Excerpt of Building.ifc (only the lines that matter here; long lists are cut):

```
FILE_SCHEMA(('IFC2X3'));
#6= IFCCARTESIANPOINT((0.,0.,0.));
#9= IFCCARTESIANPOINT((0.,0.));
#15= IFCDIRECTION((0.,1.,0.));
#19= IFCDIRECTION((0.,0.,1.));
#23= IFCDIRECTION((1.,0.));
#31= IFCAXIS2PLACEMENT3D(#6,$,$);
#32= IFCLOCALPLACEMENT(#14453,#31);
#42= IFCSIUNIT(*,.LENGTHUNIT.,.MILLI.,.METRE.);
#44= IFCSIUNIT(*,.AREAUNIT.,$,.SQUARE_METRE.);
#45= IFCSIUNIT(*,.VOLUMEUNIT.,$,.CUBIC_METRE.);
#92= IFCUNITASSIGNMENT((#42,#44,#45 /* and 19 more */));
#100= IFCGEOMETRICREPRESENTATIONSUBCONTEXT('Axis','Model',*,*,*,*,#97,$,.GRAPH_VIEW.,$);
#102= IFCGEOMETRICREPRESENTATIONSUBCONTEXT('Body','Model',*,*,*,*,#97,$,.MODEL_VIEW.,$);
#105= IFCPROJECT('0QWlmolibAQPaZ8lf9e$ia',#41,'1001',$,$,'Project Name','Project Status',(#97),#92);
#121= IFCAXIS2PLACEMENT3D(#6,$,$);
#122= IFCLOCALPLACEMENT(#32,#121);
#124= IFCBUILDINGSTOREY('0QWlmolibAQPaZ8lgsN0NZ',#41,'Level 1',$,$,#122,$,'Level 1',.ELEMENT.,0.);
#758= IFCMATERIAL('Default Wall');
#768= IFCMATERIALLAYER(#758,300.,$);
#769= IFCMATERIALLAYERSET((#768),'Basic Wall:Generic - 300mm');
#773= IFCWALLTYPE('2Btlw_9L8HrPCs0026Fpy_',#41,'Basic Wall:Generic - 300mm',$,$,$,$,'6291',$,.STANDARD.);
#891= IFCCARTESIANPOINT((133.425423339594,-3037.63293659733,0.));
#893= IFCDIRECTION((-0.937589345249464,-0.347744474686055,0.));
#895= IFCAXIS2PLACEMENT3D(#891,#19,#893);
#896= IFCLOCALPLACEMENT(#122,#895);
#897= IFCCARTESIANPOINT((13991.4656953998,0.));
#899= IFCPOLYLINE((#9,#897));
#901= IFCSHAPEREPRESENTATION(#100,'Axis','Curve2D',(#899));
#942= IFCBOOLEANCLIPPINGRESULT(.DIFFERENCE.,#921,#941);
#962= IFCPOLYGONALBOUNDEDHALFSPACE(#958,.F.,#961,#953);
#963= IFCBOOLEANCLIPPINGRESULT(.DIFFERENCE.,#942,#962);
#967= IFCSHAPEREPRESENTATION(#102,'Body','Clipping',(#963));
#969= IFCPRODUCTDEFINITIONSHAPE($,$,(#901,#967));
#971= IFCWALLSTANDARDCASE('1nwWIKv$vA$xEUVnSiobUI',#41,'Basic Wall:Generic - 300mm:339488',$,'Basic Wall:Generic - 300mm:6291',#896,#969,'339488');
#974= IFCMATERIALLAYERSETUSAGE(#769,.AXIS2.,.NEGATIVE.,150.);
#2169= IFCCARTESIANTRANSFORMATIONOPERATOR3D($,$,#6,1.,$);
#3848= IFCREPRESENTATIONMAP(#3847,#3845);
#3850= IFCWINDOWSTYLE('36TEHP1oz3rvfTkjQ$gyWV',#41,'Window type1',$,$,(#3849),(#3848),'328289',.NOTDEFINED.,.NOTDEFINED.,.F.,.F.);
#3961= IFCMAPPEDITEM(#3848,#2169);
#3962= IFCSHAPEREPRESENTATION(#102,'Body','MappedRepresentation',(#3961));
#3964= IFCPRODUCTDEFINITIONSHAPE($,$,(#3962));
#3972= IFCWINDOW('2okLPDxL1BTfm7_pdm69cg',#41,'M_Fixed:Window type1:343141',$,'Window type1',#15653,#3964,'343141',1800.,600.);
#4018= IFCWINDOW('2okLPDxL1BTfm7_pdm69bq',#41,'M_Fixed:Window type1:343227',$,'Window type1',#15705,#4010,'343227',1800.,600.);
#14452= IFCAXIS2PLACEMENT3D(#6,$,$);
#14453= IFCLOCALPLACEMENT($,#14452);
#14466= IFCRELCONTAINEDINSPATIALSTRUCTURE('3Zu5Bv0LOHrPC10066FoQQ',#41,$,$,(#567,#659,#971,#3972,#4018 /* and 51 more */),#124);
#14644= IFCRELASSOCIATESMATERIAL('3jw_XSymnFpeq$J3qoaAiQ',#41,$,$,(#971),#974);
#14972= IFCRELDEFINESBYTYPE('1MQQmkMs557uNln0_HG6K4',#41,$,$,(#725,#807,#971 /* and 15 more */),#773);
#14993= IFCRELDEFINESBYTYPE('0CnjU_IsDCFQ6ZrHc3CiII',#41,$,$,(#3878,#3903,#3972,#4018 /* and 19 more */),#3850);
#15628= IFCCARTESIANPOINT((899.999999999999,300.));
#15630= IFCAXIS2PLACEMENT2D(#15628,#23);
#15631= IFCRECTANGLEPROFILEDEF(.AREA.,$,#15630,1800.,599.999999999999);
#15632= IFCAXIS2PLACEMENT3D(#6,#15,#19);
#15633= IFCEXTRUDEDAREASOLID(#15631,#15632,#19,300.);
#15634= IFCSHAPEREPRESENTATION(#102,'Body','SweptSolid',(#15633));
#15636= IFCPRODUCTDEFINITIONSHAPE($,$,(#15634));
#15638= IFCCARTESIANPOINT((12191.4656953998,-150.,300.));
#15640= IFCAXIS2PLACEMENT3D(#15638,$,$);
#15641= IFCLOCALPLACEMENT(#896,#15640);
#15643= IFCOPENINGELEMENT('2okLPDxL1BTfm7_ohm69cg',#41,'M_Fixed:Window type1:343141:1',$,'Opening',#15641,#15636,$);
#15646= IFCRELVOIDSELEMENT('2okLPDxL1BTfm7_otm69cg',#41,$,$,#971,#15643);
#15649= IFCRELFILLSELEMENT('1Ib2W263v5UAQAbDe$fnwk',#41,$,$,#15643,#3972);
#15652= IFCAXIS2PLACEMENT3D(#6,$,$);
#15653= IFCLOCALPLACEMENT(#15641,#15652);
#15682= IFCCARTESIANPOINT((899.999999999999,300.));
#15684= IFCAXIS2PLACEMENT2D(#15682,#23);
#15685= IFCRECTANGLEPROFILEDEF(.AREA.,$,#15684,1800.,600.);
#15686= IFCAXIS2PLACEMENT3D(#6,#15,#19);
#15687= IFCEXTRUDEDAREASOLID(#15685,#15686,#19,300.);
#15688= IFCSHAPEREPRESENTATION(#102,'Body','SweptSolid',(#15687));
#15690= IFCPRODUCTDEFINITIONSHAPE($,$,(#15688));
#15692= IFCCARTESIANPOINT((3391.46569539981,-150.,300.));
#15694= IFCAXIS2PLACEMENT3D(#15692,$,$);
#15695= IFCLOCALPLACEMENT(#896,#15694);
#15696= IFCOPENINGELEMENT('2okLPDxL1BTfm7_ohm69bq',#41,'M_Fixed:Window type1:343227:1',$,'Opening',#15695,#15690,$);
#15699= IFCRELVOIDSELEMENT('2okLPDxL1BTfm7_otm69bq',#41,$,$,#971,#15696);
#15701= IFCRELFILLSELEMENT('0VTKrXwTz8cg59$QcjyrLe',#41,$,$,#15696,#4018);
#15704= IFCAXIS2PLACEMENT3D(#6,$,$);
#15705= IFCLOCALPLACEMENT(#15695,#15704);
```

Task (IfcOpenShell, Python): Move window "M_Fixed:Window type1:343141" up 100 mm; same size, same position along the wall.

```python
import numpy as np
import ifcopenshell
import ifcopenshell.api.geometry
import ifcopenshell.util.placement
import ifcopenshell.util.unit

model = ifcopenshell.open("Building.ifc")
unit_scale = ifcopenshell.util.unit.calculate_unit_scale(model)

window = model.by_guid("2okLPDxL1BTfm7_pdm69cg")
opening = window.FillsVoids[0].RelatingOpeningElement
dz = 0.1 / unit_scale

shift = np.array([0.0, 0.0, dz])
# The window is placed relative to its opening, so it follows when the opening moves.
matrix = ifcopenshell.util.placement.get_local_placement(opening.ObjectPlacement)
matrix[:3, 3] += shift
ifcopenshell.api.geometry.edit_object_placement(
    model, product=opening, matrix=matrix, is_si=False, should_transform_children=True
)

print(f"moved by {dz * unit_scale:+.3f} m")

model.write("Building_rev.ifc")
```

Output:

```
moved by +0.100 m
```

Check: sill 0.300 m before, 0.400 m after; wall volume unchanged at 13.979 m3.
